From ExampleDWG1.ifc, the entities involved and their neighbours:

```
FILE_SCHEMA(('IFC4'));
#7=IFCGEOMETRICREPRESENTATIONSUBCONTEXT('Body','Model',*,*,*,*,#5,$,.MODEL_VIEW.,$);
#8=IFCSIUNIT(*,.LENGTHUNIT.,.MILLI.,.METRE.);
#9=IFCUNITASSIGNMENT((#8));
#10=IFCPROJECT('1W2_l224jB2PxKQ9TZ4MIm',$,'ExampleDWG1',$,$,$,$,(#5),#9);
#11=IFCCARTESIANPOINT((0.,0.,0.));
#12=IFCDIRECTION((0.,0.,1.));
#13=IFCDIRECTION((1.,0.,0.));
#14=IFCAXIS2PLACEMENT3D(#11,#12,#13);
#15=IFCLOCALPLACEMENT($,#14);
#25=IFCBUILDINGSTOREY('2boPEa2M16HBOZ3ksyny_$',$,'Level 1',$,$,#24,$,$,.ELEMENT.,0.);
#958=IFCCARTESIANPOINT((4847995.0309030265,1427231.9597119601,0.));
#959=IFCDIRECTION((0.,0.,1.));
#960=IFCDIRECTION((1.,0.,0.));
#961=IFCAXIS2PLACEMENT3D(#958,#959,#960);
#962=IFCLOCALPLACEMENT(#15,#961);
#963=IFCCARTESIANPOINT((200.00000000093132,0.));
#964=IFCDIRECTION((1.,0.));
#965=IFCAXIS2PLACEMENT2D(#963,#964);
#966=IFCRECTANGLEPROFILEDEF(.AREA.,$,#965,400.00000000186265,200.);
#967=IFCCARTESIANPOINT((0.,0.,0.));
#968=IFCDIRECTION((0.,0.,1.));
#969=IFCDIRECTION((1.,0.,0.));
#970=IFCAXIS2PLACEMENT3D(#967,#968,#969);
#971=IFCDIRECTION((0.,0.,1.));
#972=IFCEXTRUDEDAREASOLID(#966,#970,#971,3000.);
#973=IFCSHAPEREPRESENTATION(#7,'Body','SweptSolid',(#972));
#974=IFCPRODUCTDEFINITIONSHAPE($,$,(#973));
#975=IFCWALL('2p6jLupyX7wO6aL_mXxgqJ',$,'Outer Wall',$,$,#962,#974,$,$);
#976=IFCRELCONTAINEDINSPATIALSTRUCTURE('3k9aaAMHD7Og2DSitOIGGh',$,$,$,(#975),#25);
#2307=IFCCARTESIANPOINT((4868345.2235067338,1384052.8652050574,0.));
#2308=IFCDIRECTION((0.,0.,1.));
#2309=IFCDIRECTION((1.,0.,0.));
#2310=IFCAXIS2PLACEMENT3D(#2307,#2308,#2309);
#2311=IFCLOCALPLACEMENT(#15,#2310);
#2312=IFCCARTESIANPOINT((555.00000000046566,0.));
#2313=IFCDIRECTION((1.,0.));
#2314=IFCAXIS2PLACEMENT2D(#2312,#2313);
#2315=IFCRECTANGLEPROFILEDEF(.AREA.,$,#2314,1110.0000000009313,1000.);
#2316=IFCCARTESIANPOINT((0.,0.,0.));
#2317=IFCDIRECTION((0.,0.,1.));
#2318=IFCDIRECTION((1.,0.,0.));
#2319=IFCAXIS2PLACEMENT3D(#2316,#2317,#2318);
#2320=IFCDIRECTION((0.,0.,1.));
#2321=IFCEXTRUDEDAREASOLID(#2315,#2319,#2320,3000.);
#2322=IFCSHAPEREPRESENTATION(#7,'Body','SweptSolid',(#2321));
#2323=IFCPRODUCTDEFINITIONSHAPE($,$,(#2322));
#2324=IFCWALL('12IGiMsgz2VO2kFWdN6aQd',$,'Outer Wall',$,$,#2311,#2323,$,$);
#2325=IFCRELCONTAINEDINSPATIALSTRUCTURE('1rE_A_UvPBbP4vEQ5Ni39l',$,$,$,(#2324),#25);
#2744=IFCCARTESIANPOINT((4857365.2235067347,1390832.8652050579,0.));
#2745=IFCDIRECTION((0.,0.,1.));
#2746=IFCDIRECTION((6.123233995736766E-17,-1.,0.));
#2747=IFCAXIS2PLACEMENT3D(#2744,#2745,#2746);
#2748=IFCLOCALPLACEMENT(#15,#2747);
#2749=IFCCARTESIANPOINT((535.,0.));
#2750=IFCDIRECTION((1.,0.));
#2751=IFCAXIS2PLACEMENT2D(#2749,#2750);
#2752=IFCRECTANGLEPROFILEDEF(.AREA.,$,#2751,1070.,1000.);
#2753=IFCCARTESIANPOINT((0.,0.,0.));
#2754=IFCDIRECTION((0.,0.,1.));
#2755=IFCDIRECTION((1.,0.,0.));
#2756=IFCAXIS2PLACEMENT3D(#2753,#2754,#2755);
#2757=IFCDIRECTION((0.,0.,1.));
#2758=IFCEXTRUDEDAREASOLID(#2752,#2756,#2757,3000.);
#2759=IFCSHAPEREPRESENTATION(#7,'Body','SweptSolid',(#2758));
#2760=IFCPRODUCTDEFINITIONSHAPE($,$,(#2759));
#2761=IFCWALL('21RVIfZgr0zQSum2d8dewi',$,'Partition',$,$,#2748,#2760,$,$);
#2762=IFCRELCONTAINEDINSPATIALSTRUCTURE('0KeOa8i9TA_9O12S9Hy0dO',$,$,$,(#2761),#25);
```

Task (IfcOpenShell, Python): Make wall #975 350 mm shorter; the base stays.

```python
import ifcopenshell
import ifcopenshell.geom
import ifcopenshell.util.representation
import ifcopenshell.util.shape
import ifcopenshell.util.unit

model = ifcopenshell.open("ExampleDWG1.ifc")
unit_scale = ifcopenshell.util.unit.calculate_unit_scale(model)
settings = ifcopenshell.geom.settings()


def volume(element):
    """Net volume in cubic metres, openings subtracted."""
    shape = ifcopenshell.geom.create_shape(settings, element)
    return ifcopenshell.util.shape.get_volume(shape.geometry)


wall = model.by_guid("2p6jLupyX7wO6aL_mXxgqJ")
before = volume(wall)

body = ifcopenshell.util.representation.get_representation(wall, "Model", "Body")
solid = body.Items[0]
old_height = solid.Depth
solid.Depth -= 0.35 / unit_scale
after = volume(wall)

print(f"height {old_height:g} -> {solid.Depth:g}, volume {before:.3f} -> {after:.3f} m3")

model.write("ExampleDWG1-out.ifc")
```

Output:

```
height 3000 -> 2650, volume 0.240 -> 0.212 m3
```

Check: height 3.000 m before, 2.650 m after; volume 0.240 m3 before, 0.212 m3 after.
